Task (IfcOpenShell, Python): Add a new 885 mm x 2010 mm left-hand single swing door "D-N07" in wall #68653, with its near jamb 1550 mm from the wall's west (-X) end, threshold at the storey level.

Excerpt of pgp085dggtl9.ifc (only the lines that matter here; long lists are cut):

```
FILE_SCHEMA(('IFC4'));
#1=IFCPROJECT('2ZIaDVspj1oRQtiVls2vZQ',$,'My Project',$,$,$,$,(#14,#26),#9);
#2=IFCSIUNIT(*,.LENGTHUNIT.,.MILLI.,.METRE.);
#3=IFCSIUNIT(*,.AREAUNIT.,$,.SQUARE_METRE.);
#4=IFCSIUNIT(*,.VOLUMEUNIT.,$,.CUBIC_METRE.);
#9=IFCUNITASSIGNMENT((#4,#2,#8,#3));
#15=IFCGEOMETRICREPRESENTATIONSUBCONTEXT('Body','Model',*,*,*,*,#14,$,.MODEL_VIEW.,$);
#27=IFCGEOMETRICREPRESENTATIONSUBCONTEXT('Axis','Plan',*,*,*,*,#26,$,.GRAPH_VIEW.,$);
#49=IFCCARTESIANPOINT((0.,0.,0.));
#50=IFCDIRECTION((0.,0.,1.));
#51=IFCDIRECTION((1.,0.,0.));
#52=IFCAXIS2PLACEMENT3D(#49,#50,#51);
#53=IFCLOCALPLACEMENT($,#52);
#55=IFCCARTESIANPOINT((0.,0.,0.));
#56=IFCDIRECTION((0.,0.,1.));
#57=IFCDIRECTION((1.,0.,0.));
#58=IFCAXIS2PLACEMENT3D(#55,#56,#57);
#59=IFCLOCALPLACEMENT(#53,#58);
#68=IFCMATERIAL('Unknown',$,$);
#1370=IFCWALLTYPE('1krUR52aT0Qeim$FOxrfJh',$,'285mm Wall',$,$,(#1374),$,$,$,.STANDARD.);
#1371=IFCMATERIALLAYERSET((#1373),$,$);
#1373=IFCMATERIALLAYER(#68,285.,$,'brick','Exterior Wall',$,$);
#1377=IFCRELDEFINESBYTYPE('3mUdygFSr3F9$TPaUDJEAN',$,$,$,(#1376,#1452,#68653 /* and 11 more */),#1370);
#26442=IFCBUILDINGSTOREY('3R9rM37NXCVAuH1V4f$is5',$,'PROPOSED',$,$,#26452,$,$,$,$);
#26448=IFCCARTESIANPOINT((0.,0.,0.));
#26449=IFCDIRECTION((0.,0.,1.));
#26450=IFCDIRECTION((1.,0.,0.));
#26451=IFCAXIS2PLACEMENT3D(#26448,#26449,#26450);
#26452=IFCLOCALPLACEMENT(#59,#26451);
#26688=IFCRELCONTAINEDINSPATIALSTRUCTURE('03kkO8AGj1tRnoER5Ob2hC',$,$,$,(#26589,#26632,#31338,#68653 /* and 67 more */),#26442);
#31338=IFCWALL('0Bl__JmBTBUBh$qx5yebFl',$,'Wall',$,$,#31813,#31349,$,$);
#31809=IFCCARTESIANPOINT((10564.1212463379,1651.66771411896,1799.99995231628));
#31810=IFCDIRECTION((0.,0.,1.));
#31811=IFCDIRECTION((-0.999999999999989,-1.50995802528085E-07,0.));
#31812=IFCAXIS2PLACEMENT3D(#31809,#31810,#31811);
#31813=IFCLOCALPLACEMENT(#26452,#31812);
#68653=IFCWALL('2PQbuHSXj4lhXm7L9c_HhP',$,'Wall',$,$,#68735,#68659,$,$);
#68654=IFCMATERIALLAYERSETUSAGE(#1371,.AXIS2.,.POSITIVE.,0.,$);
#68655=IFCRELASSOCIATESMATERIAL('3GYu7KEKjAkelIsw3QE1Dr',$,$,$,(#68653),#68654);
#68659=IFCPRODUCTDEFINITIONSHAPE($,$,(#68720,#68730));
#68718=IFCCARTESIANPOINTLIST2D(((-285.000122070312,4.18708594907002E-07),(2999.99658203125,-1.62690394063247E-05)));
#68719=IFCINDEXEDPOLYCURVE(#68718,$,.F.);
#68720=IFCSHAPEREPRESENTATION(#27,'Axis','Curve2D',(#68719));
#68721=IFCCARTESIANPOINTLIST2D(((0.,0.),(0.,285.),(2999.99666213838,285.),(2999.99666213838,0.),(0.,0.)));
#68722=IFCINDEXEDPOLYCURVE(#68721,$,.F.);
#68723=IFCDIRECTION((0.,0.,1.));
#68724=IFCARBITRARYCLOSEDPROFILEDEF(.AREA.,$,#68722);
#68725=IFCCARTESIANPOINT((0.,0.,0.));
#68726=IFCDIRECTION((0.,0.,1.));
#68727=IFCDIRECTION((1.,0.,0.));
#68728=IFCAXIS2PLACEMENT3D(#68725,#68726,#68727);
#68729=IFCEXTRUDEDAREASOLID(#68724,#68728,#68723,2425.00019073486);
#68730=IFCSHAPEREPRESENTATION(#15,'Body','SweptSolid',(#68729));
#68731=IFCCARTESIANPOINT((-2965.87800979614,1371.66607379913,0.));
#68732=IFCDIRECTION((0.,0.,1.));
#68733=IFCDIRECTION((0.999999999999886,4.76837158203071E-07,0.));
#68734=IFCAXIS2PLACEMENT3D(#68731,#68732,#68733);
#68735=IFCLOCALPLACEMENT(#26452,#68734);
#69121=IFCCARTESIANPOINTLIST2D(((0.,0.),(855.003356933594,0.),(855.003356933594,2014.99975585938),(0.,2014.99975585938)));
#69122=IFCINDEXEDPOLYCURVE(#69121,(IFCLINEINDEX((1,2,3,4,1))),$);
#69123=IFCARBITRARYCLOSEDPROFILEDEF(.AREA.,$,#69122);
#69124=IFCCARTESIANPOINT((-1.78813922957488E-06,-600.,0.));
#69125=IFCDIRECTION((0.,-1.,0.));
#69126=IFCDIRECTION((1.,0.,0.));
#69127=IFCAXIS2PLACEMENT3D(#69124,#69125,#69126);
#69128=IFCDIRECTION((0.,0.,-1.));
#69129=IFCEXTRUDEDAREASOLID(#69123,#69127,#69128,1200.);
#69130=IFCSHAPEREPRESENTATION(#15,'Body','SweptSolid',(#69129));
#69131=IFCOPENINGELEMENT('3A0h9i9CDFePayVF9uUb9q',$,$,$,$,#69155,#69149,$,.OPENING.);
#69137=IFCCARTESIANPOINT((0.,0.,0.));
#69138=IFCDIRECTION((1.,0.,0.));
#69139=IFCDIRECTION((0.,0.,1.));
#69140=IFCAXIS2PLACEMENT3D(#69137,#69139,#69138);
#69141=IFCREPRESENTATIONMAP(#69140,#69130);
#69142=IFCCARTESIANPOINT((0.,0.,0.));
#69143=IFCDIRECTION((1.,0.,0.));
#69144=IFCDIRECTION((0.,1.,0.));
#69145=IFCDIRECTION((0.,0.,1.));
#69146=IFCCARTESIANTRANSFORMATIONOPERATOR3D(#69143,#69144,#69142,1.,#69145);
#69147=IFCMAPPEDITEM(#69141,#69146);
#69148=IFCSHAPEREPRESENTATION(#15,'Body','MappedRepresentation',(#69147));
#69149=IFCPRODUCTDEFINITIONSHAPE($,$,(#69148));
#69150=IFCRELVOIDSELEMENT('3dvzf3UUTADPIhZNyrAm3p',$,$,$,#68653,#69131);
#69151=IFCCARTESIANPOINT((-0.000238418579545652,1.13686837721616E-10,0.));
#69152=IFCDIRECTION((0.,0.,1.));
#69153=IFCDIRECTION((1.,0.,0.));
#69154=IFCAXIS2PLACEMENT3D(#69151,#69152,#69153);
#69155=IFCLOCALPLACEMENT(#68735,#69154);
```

```python
import numpy as np
import ifcopenshell
import ifcopenshell.api.feature
import ifcopenshell.api.geometry
import ifcopenshell.api.root
import ifcopenshell.api.spatial
import ifcopenshell.geom
import ifcopenshell.util.element
import ifcopenshell.util.placement
import ifcopenshell.util.representation
import ifcopenshell.util.shape
import ifcopenshell.util.unit

model = ifcopenshell.open("pgp085dggtl9.ifc")
unit_scale = ifcopenshell.util.unit.calculate_unit_scale(model)
settings = ifcopenshell.geom.settings()


def volume(element):
    """Net volume in cubic metres, openings subtracted."""
    shape = ifcopenshell.geom.create_shape(settings, element)
    return ifcopenshell.util.shape.get_volume(shape.geometry)


wall = model.by_id(68653)
storey = ifcopenshell.util.element.get_container(wall, ifc_class="IfcBuildingStorey")
context = ifcopenshell.util.representation.get_context(model, "Model", "Body", "MODEL_VIEW")
before = volume(wall)

width, height, from_end, sill = 0.885, 2.01, 1.55, 0.0  # metres

# The wall runs along its own X axis, and the end named is its -X end.
wall_shape = ifcopenshell.geom.create_shape(settings, wall)
x, y, z = ifcopenshell.util.shape.get_vertices(wall_shape.geometry).T
start = x.min() + from_end
face, thickness = float(y.min()), float(y.max() - y.min())
wall_matrix = ifcopenshell.util.placement.get_local_placement(wall.ObjectPlacement)
level = ifcopenshell.util.placement.get_local_placement(storey.ObjectPlacement)[2, 3]


def in_wall(x, y):
    """Placement at x, y metres in the wall's axes, at sill height."""
    matrix = wall_matrix.copy()
    matrix[:, 3] = wall_matrix @ np.array([x / unit_scale, y / unit_scale, 0.0, 1.0])
    matrix[2, 3] = level + sill / unit_scale
    return matrix


# Opening: a box that overshoots both wall faces by 50 mm.
opening = ifcopenshell.api.root.create_entity(model, ifc_class="IfcOpeningElement", predefined_type="OPENING")
box = ifcopenshell.api.geometry.add_wall_representation(
    model, context=context, length=width, height=height, thickness=thickness + 0.1
)
ifcopenshell.api.geometry.assign_representation(model, product=opening, representation=box)
ifcopenshell.api.geometry.edit_object_placement(model, product=opening, matrix=in_wall(start, face - 0.05), is_si=False)
ifcopenshell.api.feature.add_feature(model, feature=opening, element=wall)

door = ifcopenshell.api.root.create_entity(model, ifc_class="IfcDoor", name="D-N07", predefined_type="DOOR")
door.OverallWidth, door.OverallHeight = width / unit_scale, height / unit_scale
door.OperationType = "SINGLE_SWING_LEFT"
body = ifcopenshell.api.geometry.add_door_representation(
    model,
    context=context,
    overall_width=door.OverallWidth,
    overall_height=door.OverallHeight,
    operation_type="SINGLE_SWING_LEFT",
    lining_properties={"LiningDepth": thickness / unit_scale, "ThresholdDepth": thickness / unit_scale},
)
ifcopenshell.api.geometry.assign_representation(model, product=door, representation=body)
ifcopenshell.api.spatial.assign_container(model, products=[door], relating_structure=storey)
ifcopenshell.api.feature.add_filling(model, opening=opening, element=door)

# The lining spans the wall, so the door starts at the wall face.
ifcopenshell.api.geometry.edit_object_placement(model, product=door, matrix=in_wall(start, face), is_si=False)

after = volume(wall)

print(f"wall volume {before:.3f} -> {after:.3f} m3")

model.write("pgp085dggtl9_rev.ifc")
```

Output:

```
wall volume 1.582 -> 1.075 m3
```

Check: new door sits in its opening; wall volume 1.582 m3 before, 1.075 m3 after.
